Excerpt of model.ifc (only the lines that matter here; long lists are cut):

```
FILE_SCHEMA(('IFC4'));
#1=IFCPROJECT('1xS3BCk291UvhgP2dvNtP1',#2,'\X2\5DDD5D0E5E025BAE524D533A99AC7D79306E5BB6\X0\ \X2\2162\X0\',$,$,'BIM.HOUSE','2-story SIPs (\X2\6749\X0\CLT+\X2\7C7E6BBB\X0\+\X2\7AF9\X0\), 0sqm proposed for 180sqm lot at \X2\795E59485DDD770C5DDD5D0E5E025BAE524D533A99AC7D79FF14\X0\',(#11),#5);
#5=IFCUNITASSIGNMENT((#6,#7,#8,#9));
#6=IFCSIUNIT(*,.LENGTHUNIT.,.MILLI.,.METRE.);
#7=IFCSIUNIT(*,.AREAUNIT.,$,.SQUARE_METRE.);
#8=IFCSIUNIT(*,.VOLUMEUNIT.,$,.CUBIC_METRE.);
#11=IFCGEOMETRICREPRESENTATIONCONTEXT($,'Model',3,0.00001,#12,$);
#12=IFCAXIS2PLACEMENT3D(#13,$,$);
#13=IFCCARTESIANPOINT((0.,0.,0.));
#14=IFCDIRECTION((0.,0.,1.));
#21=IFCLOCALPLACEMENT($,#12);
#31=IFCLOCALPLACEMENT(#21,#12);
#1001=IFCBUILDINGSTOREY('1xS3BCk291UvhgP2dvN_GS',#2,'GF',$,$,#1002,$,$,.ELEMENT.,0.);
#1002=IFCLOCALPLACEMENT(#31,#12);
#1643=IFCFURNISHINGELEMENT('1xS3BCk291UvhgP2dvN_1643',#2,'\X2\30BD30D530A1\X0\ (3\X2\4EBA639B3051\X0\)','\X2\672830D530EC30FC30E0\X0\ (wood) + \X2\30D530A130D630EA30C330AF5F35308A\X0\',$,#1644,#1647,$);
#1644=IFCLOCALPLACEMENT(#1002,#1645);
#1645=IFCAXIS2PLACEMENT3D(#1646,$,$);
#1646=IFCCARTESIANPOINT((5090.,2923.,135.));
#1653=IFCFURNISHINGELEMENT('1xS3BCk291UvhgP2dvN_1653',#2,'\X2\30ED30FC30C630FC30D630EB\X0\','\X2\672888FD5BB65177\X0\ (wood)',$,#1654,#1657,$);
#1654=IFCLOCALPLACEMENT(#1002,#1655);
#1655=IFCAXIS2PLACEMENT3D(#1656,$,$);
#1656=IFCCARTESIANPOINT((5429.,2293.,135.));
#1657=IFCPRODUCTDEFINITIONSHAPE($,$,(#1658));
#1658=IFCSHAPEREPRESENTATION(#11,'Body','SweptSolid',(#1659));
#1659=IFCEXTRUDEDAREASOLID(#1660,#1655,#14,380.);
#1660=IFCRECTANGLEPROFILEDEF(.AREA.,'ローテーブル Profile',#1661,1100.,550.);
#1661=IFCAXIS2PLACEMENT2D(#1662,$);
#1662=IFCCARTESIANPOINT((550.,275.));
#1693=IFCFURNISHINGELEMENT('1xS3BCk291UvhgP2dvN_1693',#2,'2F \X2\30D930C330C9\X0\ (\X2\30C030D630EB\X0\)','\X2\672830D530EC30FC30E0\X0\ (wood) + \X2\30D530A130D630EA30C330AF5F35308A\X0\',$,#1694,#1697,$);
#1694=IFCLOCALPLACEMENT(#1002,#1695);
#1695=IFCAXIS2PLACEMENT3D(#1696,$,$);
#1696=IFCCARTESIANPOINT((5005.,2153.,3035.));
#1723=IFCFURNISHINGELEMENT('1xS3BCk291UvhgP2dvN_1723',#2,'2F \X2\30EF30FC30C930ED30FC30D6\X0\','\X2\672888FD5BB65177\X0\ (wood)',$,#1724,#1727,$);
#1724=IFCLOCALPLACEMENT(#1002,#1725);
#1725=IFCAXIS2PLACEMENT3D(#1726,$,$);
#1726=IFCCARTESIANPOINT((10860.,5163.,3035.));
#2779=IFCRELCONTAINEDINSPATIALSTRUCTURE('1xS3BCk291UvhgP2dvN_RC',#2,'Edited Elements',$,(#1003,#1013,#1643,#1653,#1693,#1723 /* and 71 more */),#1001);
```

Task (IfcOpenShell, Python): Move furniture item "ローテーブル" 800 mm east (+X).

```python
import ifcopenshell
import ifcopenshell.api.geometry
import ifcopenshell.util.placement
import ifcopenshell.util.unit

model = ifcopenshell.open("model.ifc")
unit_scale = ifcopenshell.util.unit.calculate_unit_scale(model)

item = model.by_id(1653)
matrix = ifcopenshell.util.placement.get_local_placement(item.ObjectPlacement)
matrix[0, 3] += 0.8 / unit_scale
ifcopenshell.api.geometry.edit_object_placement(model, product=item, matrix=matrix, is_si=False)

print(ifcopenshell.util.placement.get_local_placement(item.ObjectPlacement).round(3) + 0.0)

model.write("model_edited.ifc")
```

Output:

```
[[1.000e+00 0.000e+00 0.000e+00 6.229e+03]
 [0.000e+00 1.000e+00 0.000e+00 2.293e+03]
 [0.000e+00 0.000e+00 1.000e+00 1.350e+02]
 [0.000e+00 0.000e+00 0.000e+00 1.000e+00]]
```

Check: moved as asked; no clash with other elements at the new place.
